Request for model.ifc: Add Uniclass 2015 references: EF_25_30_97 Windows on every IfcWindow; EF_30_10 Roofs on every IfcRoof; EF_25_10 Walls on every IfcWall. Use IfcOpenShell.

First a look at what the model holds.

```python
import ifcopenshell

model = ifcopenshell.open("model.ifc")
print(model.schema)
print("classifications:", [c.Name for c in model.by_type("IfcClassification")])
for ifc_class in ("IfcDoor", "IfcRoof", "IfcStair", "IfcWall", "IfcWindow"):
    print(ifc_class, len(model.by_type(ifc_class)))
```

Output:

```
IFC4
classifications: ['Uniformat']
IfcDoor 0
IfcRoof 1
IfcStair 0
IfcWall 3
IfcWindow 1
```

```python
import ifcopenshell
import ifcopenshell.api.classification

model = ifcopenshell.open("model.ifc")

system = ifcopenshell.api.classification.add_classification(model, classification="Uniclass 2015")

codes = {
    "IfcWindow": ("EF_25_30_97", "Windows"),
    "IfcRoof": ("EF_30_10", "Roofs"),
    "IfcWall": ("EF_25_10", "Walls"),
}
for ifc_class, (code, name) in codes.items():
    products = model.by_type(ifc_class)
    ifcopenshell.api.classification.add_reference(
        model, products=products, classification=system, identification=code, name=name
    )
    print(code, len(products))

model.write("model-out.ifc")
```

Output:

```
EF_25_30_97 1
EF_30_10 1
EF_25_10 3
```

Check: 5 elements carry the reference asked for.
